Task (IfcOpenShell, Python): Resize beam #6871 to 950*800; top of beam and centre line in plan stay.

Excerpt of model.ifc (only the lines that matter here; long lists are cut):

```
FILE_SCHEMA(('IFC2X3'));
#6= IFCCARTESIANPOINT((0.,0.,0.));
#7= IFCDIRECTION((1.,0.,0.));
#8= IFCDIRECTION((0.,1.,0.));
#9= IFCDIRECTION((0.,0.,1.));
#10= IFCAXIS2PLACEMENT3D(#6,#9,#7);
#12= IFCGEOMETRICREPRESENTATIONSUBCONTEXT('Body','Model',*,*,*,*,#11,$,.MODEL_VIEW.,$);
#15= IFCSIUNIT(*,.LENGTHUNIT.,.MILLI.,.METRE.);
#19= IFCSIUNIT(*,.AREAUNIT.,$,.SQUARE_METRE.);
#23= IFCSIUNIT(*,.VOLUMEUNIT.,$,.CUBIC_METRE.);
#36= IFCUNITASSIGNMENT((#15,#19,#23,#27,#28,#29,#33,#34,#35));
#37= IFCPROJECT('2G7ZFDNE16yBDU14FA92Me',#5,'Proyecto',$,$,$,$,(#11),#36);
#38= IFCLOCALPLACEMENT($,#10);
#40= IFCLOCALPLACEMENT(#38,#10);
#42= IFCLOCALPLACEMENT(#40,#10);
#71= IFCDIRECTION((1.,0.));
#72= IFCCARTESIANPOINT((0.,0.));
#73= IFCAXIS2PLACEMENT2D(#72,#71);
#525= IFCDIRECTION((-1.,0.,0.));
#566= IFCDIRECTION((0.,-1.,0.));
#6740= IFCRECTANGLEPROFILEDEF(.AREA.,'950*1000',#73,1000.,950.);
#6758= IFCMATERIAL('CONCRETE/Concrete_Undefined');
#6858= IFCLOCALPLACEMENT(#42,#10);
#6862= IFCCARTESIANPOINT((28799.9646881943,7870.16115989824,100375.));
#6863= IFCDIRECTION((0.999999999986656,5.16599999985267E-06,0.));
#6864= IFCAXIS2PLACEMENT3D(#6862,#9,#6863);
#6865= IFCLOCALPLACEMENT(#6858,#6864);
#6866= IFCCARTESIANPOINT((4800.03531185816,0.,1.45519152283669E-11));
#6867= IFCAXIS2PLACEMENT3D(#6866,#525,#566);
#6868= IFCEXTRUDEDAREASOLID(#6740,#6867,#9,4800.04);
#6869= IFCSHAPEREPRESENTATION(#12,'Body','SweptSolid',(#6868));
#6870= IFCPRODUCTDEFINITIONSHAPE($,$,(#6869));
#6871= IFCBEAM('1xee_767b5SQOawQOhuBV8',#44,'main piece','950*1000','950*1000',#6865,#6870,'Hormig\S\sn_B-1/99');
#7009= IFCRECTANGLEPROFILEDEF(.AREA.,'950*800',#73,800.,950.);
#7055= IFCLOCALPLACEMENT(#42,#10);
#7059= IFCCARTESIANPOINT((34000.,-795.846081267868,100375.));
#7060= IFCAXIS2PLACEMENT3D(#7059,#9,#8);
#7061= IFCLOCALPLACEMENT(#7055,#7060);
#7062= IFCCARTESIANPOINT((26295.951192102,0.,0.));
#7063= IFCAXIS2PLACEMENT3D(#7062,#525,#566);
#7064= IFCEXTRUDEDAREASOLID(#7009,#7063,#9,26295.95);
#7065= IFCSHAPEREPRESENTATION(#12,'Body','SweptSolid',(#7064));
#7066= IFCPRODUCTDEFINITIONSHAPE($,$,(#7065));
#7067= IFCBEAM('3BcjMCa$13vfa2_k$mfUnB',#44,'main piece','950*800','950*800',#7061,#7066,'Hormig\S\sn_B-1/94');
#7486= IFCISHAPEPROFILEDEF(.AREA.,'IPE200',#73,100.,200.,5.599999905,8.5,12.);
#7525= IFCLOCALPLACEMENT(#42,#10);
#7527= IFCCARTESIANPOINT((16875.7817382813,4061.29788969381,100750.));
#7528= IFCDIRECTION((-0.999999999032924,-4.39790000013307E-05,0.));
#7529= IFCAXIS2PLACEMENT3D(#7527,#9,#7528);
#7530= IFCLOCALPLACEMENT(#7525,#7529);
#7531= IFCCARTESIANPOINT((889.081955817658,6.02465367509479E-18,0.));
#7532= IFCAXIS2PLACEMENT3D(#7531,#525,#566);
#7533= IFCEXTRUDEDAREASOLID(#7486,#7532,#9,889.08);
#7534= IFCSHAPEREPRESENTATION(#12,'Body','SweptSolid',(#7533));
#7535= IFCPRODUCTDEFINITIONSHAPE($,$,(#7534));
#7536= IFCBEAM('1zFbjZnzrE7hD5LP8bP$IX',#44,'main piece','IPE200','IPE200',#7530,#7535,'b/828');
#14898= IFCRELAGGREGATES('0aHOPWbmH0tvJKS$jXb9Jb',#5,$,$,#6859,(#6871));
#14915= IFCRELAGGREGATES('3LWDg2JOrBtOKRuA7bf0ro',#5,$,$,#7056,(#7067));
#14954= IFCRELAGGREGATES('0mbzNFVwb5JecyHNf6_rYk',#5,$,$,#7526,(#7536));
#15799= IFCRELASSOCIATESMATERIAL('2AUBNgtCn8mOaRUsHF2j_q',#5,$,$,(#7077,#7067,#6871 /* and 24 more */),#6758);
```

```python
import ifcopenshell
import ifcopenshell.util.element
import ifcopenshell.util.representation

model = ifcopenshell.open("model.ifc")

member = model.by_id(6871)
source = next(p for p in model.by_type("IfcRectangleProfileDef") if p.ProfileName == "950*800")

body = ifcopenshell.util.representation.get_representation(member, "Model", "Body")
solid = body.Items[0]
old_profile = solid.SweptArea

# Copy the section's sizes but keep this member's own profile position.
profile = ifcopenshell.util.element.copy(model, source)
# Profiles are centred, so shift by half the change in depth to hold the top.
shift = (old_profile.YDim - profile.YDim) / 2
x, y = old_profile.Position.Location.Coordinates
up = (0.0, 1.0)  # upwards, in the solid's own plane
location = model.createIfcCartesianPoint((x + up[0] * shift, y + up[1] * shift))
profile.Position = model.createIfcAxis2Placement2D(location, old_profile.Position.RefDirection)
solid.SweptArea = profile
if not model.get_total_inverses(old_profile):
    ifcopenshell.util.element.remove_deep2(model, old_profile)
member.Description = member.Description.replace("950*1000", "950*800")
member.ObjectType = member.ObjectType.replace("950*1000", "950*800")

print(solid.SweptArea)

model.write("model-out.ifc")
```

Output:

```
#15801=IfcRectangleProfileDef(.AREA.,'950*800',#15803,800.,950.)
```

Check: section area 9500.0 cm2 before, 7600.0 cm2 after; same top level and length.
